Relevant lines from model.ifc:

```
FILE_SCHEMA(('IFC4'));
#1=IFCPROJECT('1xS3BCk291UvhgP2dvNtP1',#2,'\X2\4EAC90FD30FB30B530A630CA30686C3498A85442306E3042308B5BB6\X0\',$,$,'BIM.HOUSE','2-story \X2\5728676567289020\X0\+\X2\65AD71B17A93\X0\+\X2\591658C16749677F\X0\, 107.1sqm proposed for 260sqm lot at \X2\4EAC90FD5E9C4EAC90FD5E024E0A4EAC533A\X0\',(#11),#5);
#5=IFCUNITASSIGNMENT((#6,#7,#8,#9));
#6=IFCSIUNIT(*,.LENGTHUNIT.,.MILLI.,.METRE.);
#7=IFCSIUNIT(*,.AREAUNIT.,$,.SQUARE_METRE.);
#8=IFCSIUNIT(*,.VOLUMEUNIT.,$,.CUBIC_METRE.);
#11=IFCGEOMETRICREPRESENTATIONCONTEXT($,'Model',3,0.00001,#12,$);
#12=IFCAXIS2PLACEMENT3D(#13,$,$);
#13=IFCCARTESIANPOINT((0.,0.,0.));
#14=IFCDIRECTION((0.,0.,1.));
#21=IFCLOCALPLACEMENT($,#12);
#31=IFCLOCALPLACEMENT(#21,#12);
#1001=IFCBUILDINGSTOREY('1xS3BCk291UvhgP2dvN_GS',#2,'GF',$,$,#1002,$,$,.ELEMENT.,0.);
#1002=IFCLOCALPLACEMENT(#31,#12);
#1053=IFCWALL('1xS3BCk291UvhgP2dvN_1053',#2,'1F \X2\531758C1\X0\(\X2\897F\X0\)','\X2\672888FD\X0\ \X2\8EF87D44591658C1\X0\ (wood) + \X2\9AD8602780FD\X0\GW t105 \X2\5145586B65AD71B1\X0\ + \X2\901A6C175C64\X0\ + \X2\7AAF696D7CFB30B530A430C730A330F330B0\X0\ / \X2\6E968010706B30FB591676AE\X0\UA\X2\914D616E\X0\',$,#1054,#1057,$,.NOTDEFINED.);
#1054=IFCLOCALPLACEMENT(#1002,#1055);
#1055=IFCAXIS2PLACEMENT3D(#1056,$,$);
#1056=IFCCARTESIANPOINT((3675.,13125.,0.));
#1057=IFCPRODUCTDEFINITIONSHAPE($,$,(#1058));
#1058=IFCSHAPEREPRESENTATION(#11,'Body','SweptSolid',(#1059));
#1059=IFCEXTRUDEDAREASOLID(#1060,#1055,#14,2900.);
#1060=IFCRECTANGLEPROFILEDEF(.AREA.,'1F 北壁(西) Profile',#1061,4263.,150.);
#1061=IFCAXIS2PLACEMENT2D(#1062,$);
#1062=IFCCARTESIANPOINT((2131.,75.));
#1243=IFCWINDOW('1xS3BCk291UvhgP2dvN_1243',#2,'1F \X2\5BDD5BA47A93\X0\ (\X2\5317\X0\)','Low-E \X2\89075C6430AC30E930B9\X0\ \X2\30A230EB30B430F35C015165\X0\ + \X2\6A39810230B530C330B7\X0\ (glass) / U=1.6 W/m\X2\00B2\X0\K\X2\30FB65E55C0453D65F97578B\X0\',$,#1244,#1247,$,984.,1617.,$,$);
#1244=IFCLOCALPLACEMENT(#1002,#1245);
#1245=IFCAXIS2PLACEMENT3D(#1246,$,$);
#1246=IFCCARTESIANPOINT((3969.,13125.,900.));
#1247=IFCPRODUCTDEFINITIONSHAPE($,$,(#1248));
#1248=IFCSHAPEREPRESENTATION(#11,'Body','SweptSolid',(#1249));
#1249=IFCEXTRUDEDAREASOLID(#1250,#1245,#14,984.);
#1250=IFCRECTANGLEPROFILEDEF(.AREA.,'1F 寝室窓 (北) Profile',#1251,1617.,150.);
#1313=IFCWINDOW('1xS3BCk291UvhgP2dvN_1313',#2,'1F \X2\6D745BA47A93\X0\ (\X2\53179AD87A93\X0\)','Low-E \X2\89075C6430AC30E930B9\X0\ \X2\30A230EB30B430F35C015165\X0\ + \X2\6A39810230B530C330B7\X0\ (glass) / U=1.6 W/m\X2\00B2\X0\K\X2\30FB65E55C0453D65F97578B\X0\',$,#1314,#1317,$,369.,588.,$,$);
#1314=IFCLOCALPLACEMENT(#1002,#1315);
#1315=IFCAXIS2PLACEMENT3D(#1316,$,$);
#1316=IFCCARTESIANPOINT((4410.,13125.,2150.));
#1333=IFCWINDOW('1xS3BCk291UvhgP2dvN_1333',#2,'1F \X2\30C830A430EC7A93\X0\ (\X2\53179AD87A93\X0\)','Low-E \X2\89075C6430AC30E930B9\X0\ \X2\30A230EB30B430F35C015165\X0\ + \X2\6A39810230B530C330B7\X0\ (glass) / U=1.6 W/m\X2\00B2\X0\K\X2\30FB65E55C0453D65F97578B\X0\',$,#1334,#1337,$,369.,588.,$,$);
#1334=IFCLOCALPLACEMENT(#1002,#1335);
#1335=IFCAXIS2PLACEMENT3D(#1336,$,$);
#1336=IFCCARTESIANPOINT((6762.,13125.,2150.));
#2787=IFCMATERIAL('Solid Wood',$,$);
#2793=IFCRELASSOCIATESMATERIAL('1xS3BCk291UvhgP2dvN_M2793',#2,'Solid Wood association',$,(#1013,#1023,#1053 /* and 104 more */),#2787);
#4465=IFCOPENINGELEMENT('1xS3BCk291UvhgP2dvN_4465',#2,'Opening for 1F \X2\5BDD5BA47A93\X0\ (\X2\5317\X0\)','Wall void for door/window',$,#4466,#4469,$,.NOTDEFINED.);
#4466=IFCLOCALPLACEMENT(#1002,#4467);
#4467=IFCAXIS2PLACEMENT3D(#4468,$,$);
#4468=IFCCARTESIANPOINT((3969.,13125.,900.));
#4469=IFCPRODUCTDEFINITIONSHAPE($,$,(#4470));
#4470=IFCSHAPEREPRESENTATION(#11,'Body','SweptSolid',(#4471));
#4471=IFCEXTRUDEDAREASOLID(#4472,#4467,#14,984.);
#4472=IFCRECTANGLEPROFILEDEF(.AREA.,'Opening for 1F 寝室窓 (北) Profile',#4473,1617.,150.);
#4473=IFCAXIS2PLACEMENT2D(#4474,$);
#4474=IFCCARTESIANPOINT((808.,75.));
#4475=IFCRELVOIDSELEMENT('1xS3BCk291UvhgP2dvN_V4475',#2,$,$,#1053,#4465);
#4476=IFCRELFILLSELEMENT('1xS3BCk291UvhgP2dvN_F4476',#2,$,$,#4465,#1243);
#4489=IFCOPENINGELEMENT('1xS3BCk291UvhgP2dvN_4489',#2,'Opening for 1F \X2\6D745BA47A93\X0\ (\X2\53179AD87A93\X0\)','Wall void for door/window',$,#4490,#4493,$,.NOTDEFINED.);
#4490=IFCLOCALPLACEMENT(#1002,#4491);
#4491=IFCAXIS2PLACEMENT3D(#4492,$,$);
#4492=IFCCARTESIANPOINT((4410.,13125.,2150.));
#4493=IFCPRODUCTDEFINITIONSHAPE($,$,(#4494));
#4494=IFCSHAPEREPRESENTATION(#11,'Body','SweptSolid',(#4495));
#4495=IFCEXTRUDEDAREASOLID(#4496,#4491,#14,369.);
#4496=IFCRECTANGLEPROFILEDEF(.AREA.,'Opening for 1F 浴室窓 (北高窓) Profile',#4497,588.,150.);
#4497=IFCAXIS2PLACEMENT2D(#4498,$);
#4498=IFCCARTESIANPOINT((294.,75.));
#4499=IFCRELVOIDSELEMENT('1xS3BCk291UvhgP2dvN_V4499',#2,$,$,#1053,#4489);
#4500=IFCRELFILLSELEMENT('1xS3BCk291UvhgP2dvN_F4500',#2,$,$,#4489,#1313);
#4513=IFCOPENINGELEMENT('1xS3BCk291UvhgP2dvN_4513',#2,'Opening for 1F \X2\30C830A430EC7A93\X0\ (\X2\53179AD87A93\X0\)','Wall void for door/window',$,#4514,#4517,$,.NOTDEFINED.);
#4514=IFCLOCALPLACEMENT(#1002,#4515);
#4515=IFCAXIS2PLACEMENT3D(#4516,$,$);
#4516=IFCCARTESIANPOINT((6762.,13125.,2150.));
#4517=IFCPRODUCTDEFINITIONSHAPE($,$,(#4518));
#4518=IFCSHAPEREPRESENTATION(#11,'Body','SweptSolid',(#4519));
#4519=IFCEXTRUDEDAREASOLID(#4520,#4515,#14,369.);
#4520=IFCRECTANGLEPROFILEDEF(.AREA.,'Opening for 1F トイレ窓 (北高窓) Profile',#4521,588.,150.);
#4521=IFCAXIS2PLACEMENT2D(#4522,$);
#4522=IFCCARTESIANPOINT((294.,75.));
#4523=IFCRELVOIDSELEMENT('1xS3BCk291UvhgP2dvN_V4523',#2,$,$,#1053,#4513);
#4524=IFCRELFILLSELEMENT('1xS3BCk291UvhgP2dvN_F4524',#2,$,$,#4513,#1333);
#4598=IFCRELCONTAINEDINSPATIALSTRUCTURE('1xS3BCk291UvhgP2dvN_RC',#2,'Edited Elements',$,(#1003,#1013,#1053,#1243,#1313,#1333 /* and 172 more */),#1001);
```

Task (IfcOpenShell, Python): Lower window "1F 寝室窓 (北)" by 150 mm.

```python
import numpy as np
import ifcopenshell
import ifcopenshell.api.geometry
import ifcopenshell.util.placement
import ifcopenshell.util.unit

model = ifcopenshell.open("model.ifc")
unit_scale = ifcopenshell.util.unit.calculate_unit_scale(model)

window = model.by_guid("1xS3BCk291UvhgP2dvN_1243")
opening = window.FillsVoids[0].RelatingOpeningElement
dz = -150.0

shift = np.array([0.0, 0.0, dz])
# The window is not placed relative to its opening, so move both.
for product in (opening, window):
    matrix = ifcopenshell.util.placement.get_local_placement(product.ObjectPlacement)
    matrix[:3, 3] += shift
    ifcopenshell.api.geometry.edit_object_placement(model, product=product, matrix=matrix, is_si=False)

print(f"moved by {dz * unit_scale:+.3f} m")

model.write("model_edited.ifc")
```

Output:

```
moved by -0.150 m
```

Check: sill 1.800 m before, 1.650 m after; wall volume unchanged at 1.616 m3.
